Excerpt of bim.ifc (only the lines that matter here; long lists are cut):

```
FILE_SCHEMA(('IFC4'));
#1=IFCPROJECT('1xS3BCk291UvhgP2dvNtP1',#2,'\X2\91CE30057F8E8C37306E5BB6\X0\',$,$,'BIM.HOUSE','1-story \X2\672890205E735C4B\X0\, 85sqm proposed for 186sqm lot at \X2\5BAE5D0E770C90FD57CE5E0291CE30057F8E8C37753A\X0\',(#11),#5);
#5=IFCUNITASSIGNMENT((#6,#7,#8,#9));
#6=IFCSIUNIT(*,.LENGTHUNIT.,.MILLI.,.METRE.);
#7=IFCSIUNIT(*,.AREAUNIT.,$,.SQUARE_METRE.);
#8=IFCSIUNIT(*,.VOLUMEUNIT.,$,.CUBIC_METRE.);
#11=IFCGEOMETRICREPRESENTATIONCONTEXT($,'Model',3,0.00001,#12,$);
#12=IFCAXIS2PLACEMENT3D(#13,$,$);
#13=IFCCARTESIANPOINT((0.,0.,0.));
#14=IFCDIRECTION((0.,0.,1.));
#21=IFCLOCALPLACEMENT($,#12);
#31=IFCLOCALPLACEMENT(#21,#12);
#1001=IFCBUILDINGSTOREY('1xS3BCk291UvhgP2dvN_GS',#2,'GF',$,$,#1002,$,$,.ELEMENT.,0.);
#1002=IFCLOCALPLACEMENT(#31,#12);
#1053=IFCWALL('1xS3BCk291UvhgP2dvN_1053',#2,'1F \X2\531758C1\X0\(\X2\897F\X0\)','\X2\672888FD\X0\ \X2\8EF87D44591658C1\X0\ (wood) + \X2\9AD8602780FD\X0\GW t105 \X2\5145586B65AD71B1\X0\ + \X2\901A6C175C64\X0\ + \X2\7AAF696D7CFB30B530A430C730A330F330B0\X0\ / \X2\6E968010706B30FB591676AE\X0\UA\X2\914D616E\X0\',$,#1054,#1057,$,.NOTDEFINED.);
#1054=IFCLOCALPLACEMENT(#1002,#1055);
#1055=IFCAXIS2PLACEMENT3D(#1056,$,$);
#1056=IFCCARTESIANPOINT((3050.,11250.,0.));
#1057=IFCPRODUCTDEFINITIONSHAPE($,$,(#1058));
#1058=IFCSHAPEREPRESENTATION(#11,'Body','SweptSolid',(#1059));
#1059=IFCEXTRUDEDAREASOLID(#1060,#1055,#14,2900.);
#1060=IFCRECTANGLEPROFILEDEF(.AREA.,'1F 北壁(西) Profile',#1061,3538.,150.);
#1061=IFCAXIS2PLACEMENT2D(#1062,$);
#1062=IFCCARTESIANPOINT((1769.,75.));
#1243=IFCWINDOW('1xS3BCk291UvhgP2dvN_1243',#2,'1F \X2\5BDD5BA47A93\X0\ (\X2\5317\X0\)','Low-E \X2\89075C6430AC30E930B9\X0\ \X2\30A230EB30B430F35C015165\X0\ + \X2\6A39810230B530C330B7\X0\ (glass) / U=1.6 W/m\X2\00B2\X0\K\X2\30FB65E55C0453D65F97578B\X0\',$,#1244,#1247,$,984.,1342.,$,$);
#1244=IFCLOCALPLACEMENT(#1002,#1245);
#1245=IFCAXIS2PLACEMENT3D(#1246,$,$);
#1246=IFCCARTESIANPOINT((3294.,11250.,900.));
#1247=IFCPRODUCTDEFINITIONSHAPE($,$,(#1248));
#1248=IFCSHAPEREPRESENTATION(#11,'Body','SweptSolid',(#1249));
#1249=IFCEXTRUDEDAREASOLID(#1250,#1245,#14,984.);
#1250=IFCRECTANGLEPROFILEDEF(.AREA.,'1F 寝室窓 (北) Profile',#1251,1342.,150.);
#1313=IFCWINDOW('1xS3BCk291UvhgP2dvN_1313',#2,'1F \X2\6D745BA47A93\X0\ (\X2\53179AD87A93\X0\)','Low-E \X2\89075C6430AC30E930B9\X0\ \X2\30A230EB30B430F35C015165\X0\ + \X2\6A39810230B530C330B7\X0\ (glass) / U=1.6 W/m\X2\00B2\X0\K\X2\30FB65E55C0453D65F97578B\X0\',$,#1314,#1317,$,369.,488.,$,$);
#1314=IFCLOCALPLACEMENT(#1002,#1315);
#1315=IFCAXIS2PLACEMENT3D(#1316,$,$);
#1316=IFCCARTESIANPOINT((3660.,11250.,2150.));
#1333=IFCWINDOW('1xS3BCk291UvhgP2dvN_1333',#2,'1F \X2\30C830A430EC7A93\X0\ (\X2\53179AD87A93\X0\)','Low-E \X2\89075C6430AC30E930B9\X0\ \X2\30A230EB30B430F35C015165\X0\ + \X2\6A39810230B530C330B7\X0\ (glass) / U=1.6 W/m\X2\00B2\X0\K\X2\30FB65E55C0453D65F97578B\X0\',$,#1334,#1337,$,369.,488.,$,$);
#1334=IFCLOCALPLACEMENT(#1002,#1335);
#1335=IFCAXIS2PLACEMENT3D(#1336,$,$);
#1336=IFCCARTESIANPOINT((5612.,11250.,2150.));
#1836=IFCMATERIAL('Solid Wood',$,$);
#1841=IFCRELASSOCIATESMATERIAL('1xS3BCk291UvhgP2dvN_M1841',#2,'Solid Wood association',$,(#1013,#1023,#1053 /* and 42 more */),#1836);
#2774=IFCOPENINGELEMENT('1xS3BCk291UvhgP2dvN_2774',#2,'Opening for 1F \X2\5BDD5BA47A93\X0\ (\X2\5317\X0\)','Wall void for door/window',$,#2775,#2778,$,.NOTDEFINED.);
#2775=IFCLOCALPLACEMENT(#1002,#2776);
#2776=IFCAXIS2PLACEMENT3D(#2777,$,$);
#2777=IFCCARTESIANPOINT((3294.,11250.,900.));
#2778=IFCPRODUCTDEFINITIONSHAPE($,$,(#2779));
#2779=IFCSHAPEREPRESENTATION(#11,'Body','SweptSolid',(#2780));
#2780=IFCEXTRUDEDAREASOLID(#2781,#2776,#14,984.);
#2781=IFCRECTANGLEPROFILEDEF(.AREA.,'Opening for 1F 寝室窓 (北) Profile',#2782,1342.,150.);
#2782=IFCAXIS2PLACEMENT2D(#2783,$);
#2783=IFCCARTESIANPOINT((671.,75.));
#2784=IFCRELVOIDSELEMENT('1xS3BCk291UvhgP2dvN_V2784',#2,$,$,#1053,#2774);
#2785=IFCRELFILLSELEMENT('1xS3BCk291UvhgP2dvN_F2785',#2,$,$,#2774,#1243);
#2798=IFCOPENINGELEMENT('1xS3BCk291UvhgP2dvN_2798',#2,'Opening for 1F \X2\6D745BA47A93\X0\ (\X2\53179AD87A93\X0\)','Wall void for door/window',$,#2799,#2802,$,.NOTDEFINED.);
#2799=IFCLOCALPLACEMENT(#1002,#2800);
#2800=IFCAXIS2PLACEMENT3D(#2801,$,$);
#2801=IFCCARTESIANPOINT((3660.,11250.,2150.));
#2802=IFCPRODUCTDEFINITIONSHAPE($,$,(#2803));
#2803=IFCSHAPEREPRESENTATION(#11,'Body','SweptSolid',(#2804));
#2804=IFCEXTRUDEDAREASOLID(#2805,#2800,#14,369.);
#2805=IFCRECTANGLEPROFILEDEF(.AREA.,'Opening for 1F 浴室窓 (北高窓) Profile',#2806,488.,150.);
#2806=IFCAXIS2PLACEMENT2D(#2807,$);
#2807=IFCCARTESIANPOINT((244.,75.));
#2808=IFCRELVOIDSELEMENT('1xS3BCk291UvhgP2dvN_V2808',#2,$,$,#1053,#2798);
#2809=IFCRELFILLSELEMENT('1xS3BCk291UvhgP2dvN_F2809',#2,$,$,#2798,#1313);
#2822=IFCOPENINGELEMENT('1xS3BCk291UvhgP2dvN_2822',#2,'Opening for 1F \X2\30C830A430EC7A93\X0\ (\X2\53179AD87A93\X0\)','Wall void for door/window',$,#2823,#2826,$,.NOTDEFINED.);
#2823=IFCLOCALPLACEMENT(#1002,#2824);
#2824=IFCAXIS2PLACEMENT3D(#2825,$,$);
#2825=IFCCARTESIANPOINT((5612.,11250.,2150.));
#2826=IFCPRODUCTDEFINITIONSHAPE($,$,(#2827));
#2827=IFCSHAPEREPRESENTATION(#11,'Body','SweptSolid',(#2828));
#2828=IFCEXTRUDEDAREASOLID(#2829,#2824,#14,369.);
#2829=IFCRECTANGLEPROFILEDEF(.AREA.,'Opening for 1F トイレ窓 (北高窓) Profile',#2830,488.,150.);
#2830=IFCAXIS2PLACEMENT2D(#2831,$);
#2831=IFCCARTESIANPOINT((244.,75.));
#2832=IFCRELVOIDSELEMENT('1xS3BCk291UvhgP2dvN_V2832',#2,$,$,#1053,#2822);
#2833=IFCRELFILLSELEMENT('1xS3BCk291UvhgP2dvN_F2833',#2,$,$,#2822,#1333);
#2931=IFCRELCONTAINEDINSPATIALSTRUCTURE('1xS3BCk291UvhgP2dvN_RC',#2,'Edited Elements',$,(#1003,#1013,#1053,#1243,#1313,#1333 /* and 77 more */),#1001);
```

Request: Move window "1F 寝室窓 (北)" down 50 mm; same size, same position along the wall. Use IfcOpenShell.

```python
import numpy as np
import ifcopenshell
import ifcopenshell.api.geometry
import ifcopenshell.util.placement
import ifcopenshell.util.unit

model = ifcopenshell.open("bim.ifc")
unit_scale = ifcopenshell.util.unit.calculate_unit_scale(model)

window = model.by_guid("1xS3BCk291UvhgP2dvN_1243")
opening = window.FillsVoids[0].RelatingOpeningElement
dz = -0.05 / unit_scale

shift = np.array([0.0, 0.0, dz])
# The window is not placed relative to its opening, so move both.
for product in (opening, window):
    matrix = ifcopenshell.util.placement.get_local_placement(product.ObjectPlacement)
    matrix[:3, 3] += shift
    ifcopenshell.api.geometry.edit_object_placement(model, product=product, matrix=matrix, is_si=False)

print(f"moved by {dz * unit_scale:+.3f} m")

model.write("bim_rev.ifc")
```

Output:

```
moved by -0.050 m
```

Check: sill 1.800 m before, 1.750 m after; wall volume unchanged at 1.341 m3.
